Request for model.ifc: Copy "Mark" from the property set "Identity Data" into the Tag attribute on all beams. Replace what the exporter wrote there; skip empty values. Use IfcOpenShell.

First a look at what the model holds.

```python
import ifcopenshell
import ifcopenshell.util.element

model = ifcopenshell.open("model.ifc")
print(model.schema)
beams = model.by_type("IfcBeam")
print(len(beams), "beams")
for e in beams[:8]:
    source = ifcopenshell.util.element.get_pset(e, "Identity Data", "Mark")
    target = e.Tag
    print(e.id(), repr(source), repr(target), sep=" | ")
```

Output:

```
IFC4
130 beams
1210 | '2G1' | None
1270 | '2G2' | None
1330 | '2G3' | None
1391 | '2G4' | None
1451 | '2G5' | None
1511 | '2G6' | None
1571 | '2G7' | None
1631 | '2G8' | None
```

```python
import ifcopenshell
import ifcopenshell.util.element

model = ifcopenshell.open("model.ifc")

count = 0
for e in model.by_type("IfcBeam"):
    value = ifcopenshell.util.element.get_pset(e, "Identity Data", "Mark")
    current = e.Tag
    if not value or not value.strip() or current == value:
        continue
    e.Tag = value
    count += 1

print(count, "beams updated")

model.write("model_updated.ifc")
```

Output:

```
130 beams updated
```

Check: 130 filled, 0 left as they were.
